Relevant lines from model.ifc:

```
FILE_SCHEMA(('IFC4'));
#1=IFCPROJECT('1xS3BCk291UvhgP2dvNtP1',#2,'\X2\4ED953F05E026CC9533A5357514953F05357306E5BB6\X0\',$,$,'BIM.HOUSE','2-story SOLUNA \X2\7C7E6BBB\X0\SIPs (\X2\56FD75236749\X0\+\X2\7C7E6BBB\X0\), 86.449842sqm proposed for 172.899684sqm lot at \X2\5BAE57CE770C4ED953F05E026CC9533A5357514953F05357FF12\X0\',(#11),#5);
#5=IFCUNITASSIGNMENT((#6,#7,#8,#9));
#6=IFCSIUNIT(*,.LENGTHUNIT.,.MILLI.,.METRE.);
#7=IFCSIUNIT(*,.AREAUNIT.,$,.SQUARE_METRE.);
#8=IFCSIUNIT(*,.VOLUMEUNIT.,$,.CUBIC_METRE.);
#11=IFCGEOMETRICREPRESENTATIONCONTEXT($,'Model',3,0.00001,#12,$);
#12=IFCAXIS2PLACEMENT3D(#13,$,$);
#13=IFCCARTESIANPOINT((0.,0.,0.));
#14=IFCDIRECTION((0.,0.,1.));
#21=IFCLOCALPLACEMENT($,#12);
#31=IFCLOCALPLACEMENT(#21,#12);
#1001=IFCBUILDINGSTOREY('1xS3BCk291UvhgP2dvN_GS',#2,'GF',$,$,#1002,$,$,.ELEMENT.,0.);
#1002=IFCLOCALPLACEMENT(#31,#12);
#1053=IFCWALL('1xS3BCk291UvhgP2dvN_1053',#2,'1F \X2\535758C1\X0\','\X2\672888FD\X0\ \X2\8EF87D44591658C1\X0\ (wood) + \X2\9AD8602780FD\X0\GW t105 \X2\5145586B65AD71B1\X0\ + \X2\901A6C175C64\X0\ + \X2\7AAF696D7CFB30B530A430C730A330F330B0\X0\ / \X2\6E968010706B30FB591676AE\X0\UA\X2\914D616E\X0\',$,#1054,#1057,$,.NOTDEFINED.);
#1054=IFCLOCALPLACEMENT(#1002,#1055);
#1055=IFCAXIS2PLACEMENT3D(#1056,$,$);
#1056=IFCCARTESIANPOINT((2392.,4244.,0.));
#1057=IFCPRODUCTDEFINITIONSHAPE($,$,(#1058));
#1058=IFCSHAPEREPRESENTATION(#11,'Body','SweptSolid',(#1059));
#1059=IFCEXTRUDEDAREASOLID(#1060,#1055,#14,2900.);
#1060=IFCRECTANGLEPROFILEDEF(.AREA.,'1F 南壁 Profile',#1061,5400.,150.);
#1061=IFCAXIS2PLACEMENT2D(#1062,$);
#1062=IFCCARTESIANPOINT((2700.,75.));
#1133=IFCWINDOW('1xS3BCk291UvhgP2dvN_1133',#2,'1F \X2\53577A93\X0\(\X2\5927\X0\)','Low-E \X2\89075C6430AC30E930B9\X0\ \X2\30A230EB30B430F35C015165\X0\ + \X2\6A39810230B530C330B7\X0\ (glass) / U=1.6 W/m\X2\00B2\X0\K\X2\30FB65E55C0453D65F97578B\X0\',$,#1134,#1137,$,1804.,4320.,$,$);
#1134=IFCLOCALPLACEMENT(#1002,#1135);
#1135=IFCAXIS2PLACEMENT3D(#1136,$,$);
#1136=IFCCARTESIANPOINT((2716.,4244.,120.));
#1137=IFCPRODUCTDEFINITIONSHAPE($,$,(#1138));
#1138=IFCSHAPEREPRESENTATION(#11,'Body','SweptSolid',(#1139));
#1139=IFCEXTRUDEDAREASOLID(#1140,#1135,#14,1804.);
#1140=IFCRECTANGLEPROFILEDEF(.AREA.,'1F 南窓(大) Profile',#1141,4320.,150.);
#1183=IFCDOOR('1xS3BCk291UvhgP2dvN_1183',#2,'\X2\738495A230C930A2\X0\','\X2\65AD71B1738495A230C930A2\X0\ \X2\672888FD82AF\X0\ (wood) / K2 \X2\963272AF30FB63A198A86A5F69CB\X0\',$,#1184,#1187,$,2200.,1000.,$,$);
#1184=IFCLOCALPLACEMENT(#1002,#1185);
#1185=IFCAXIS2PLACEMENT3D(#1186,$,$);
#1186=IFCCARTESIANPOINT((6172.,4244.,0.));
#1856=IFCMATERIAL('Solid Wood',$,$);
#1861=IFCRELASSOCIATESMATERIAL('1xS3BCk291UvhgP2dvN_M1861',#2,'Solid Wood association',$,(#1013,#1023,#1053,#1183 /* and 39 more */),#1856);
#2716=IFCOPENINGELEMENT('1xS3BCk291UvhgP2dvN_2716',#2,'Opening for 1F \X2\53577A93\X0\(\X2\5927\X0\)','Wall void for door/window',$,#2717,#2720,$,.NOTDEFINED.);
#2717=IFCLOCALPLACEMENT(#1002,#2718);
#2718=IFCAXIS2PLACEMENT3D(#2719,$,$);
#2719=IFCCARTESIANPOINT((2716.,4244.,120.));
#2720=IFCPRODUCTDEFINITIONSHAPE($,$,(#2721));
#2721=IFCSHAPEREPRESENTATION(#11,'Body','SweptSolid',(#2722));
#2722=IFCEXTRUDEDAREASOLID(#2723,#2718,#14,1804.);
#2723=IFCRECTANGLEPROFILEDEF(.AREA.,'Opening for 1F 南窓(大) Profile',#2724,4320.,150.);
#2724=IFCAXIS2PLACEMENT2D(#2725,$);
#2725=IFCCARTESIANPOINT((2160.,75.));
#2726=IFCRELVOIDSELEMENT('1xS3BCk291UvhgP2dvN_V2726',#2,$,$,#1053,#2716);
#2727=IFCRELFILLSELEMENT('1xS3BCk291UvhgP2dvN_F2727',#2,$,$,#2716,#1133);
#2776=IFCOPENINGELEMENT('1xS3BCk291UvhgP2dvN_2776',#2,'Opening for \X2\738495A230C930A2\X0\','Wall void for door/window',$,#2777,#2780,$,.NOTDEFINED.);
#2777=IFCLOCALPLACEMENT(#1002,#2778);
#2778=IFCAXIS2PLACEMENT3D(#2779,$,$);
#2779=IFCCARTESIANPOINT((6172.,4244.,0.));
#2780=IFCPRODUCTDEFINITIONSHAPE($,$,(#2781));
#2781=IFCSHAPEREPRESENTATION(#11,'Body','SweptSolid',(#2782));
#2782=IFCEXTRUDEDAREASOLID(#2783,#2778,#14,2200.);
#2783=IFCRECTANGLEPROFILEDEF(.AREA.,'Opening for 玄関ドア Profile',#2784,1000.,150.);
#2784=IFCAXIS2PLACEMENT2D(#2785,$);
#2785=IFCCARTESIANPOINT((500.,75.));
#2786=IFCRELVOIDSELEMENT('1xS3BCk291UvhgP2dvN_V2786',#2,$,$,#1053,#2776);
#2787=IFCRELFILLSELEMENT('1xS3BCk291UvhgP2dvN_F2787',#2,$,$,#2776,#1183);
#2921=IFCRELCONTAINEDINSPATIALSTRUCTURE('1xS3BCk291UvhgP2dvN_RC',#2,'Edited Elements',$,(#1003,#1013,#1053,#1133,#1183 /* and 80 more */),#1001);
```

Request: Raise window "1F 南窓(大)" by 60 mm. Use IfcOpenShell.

```python
import numpy as np
import ifcopenshell
import ifcopenshell.api.geometry
import ifcopenshell.util.placement
import ifcopenshell.util.unit

model = ifcopenshell.open("model.ifc")
unit_scale = ifcopenshell.util.unit.calculate_unit_scale(model)

window = model.by_id(1133)
opening = window.FillsVoids[0].RelatingOpeningElement
dz = 0.06 / unit_scale

shift = np.array([0.0, 0.0, dz])
# The window is not placed relative to its opening, so move both.
for product in (opening, window):
    matrix = ifcopenshell.util.placement.get_local_placement(product.ObjectPlacement)
    matrix[:3, 3] += shift
    ifcopenshell.api.geometry.edit_object_placement(model, product=product, matrix=matrix, is_si=False)

print(f"moved by {dz * unit_scale:+.3f} m")

model.write("model-out.ifc")
```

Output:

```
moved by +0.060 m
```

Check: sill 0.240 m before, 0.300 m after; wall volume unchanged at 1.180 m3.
